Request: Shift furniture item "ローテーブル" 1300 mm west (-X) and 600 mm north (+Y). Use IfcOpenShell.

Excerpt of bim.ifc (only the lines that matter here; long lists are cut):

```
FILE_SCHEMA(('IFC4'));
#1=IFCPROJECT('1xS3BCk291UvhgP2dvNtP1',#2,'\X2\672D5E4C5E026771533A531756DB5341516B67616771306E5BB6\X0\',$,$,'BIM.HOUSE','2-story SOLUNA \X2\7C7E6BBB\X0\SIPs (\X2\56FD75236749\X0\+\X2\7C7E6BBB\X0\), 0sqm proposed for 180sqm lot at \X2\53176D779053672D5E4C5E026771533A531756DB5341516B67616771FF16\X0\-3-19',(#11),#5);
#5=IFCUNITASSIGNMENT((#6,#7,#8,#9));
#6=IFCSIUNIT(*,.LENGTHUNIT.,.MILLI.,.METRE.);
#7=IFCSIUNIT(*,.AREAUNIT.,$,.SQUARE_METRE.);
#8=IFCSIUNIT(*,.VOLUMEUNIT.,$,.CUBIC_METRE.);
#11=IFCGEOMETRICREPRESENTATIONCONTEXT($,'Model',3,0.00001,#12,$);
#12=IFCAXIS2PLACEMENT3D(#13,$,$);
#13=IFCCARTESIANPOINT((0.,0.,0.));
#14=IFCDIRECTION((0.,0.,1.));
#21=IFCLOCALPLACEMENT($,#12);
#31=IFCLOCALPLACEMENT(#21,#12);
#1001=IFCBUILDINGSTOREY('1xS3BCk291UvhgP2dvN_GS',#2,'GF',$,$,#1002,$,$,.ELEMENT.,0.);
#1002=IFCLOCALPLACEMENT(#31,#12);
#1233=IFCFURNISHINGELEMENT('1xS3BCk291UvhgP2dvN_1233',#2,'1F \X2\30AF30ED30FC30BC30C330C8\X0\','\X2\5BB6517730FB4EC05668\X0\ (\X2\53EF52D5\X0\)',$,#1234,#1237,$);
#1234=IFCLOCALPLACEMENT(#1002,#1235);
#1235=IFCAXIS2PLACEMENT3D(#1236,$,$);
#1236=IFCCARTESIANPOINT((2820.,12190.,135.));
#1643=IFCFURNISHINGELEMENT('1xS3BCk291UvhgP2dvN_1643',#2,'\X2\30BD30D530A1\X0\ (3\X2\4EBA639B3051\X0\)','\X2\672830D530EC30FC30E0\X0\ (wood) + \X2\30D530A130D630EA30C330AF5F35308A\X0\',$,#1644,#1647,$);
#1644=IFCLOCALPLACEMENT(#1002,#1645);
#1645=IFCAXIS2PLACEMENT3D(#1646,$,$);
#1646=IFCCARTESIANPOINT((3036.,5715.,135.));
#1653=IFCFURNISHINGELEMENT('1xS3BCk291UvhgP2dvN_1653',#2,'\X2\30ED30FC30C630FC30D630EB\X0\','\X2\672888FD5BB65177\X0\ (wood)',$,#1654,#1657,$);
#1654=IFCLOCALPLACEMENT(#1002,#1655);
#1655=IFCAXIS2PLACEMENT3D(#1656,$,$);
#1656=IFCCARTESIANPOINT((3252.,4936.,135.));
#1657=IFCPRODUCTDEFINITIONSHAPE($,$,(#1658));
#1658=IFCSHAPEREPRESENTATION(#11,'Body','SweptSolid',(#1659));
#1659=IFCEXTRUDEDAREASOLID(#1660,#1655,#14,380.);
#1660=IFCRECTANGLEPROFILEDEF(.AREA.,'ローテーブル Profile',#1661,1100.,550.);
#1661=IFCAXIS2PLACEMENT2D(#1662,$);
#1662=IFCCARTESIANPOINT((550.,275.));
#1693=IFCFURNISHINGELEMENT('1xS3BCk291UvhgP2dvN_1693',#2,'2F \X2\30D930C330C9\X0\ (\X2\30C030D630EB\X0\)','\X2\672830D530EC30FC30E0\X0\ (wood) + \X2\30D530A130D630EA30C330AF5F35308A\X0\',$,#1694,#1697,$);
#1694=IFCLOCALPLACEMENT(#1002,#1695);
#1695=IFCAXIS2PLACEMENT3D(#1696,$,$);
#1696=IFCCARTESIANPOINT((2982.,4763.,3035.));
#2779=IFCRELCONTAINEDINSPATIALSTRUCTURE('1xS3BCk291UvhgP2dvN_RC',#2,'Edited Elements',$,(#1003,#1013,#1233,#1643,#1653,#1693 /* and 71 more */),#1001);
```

```python
import ifcopenshell
import ifcopenshell.api.geometry
import ifcopenshell.util.placement

model = ifcopenshell.open("bim.ifc")

item = model.by_id(1653)
matrix = ifcopenshell.util.placement.get_local_placement(item.ObjectPlacement)
matrix[0, 3] -= 1300.0
matrix[1, 3] += 600.0
ifcopenshell.api.geometry.edit_object_placement(model, product=item, matrix=matrix, is_si=False)

print(ifcopenshell.util.placement.get_local_placement(item.ObjectPlacement).round(3) + 0.0)

model.write("bim_rev.ifc")
```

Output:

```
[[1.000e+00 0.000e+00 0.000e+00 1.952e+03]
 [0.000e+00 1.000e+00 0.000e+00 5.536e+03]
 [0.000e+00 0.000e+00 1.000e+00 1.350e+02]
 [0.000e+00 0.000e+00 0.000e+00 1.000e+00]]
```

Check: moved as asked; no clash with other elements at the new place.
